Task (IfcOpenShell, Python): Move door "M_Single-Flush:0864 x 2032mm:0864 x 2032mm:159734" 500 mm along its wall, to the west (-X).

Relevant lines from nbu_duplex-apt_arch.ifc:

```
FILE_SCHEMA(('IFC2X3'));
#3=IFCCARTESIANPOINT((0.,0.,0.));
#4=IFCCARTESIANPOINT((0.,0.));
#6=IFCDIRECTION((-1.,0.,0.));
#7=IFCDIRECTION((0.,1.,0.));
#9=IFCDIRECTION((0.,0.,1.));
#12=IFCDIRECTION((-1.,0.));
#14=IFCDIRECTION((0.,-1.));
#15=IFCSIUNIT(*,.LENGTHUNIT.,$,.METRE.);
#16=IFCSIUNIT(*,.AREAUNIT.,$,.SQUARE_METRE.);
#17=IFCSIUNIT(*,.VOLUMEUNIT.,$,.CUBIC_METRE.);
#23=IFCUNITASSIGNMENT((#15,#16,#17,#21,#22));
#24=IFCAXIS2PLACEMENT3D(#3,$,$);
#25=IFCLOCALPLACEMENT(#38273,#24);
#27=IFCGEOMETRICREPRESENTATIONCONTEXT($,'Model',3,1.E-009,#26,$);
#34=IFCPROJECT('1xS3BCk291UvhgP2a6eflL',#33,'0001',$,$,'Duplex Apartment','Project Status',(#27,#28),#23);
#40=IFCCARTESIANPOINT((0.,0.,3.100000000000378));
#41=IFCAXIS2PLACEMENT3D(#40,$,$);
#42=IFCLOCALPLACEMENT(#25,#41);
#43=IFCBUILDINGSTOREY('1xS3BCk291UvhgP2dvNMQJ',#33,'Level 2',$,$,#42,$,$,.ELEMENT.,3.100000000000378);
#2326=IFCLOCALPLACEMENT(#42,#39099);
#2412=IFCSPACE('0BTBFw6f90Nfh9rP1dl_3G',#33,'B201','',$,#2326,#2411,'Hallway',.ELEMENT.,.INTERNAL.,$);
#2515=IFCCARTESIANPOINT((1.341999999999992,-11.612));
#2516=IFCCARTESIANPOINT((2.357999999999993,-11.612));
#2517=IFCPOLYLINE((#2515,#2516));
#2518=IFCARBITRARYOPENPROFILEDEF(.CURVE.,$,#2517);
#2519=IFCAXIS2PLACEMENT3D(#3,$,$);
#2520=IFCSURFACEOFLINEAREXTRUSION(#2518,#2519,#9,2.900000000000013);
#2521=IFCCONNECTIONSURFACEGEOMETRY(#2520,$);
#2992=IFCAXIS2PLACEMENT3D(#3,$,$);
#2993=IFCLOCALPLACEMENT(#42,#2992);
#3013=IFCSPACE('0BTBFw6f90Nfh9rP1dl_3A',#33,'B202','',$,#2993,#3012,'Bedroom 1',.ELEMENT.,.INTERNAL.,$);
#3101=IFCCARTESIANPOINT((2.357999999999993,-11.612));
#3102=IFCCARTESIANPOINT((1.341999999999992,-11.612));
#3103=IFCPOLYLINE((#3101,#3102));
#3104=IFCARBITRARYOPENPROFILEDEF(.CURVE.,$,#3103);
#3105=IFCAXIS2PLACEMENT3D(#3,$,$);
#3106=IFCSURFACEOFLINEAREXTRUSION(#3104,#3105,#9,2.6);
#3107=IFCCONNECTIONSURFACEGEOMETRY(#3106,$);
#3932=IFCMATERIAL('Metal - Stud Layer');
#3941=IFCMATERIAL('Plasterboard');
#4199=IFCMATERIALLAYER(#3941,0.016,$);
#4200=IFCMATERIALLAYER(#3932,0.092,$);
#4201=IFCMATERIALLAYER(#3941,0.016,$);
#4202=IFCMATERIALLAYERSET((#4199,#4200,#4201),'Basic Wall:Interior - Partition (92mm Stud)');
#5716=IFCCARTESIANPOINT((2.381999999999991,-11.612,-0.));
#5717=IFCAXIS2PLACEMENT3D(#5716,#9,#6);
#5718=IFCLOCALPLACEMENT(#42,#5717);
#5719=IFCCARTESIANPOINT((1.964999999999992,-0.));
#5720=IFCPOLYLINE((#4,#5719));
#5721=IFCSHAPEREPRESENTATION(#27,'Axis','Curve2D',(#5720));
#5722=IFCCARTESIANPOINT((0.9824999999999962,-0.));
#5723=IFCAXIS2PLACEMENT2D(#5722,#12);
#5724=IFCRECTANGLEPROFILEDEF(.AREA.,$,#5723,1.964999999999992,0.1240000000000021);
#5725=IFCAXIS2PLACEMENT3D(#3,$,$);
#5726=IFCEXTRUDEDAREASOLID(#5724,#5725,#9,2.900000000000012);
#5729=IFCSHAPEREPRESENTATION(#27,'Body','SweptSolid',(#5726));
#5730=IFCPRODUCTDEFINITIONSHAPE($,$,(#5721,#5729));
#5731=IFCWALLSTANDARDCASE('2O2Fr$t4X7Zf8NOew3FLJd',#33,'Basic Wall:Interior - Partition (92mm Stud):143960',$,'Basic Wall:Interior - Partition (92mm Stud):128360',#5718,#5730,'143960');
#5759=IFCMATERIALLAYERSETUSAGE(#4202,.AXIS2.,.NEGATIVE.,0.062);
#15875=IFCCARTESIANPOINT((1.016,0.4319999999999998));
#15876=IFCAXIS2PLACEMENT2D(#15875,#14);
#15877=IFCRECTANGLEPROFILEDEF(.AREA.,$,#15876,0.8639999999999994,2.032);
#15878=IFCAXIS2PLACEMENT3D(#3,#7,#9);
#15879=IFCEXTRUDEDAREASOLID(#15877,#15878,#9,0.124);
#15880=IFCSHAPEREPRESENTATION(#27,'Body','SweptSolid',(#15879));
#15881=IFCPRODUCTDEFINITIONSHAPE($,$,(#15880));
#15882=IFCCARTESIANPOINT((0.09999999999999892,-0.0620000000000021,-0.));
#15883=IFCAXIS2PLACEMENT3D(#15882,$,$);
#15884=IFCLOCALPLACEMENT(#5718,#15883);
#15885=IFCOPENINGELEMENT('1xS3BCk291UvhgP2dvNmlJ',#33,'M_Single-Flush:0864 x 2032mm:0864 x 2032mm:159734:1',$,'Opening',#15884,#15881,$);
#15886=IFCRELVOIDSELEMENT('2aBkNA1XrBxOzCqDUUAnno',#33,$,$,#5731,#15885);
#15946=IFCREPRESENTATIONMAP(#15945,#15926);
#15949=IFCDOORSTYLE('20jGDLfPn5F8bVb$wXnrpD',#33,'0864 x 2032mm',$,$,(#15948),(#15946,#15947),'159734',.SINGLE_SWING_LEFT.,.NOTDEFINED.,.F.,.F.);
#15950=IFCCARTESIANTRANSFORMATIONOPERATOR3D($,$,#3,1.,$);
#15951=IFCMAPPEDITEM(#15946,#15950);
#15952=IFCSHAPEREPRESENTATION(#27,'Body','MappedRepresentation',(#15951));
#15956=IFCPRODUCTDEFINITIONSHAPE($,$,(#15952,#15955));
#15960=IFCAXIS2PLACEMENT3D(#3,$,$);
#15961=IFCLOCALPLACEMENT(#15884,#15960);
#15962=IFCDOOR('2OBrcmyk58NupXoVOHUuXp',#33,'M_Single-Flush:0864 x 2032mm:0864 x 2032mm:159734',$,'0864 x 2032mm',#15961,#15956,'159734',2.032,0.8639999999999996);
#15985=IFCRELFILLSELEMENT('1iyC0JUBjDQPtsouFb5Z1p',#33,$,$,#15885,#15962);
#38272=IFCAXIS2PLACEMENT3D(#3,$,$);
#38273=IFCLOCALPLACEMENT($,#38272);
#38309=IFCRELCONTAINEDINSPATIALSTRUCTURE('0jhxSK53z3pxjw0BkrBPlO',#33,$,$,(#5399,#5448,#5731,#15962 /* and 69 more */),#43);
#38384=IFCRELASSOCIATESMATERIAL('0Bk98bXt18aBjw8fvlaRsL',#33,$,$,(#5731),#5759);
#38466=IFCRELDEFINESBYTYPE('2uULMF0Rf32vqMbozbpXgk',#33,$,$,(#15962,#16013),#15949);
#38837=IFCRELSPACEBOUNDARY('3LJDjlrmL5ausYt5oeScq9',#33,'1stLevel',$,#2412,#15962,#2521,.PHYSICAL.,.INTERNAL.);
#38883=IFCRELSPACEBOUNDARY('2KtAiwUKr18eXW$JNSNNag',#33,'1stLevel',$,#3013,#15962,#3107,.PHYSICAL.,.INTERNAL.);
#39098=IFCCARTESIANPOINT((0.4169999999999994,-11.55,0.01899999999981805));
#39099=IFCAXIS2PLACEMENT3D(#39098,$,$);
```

```python
import numpy as np
import ifcopenshell
import ifcopenshell.api.geometry
import ifcopenshell.util.placement

model = ifcopenshell.open("nbu_duplex-apt_arch.ifc")

door = model.by_guid("2OBrcmyk58NupXoVOHUuXp")
opening = door.FillsVoids[0].RelatingOpeningElement
wall = opening.VoidsElements[0].RelatingBuildingElement

wall_matrix = ifcopenshell.util.placement.get_local_placement(wall.ObjectPlacement)
shift = wall_matrix[:3, 0] * 0.5
before = ifcopenshell.util.placement.get_local_placement(door.ObjectPlacement)[:3, 3].copy()

# The door is placed relative to its opening, so it follows when the opening moves.
matrix = ifcopenshell.util.placement.get_local_placement(opening.ObjectPlacement)
matrix[:3, 3] += shift
ifcopenshell.api.geometry.edit_object_placement(
    model, product=opening, matrix=matrix, is_si=False, should_transform_children=True
)

# Space boundary surfaces are stored in each space's coordinates; move them too.
for rel in door.ProvidesBoundaries:
    if not rel.ConnectionGeometry:
        continue
    surface = rel.ConnectionGeometry.SurfaceOnRelatingElement
    space_matrix = ifcopenshell.util.placement.get_local_placement(rel.RelatingSpace.ObjectPlacement)
    point = np.array(surface.Position.Location.Coordinates) + space_matrix[:3, :3].T @ shift
    surface.Position = model.createIfcAxis2Placement3D(
        model.createIfcCartesianPoint(point.tolist()), surface.Position.Axis, surface.Position.RefDirection
    )

after = ifcopenshell.util.placement.get_local_placement(door.ObjectPlacement)[:3, 3]
print("door moved by", (after - before).round(3) + 0.0)

model.write("nbu_duplex-apt_arch_updated.ifc")
```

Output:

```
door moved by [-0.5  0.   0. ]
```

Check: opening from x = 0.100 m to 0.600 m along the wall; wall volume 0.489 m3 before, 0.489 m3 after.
